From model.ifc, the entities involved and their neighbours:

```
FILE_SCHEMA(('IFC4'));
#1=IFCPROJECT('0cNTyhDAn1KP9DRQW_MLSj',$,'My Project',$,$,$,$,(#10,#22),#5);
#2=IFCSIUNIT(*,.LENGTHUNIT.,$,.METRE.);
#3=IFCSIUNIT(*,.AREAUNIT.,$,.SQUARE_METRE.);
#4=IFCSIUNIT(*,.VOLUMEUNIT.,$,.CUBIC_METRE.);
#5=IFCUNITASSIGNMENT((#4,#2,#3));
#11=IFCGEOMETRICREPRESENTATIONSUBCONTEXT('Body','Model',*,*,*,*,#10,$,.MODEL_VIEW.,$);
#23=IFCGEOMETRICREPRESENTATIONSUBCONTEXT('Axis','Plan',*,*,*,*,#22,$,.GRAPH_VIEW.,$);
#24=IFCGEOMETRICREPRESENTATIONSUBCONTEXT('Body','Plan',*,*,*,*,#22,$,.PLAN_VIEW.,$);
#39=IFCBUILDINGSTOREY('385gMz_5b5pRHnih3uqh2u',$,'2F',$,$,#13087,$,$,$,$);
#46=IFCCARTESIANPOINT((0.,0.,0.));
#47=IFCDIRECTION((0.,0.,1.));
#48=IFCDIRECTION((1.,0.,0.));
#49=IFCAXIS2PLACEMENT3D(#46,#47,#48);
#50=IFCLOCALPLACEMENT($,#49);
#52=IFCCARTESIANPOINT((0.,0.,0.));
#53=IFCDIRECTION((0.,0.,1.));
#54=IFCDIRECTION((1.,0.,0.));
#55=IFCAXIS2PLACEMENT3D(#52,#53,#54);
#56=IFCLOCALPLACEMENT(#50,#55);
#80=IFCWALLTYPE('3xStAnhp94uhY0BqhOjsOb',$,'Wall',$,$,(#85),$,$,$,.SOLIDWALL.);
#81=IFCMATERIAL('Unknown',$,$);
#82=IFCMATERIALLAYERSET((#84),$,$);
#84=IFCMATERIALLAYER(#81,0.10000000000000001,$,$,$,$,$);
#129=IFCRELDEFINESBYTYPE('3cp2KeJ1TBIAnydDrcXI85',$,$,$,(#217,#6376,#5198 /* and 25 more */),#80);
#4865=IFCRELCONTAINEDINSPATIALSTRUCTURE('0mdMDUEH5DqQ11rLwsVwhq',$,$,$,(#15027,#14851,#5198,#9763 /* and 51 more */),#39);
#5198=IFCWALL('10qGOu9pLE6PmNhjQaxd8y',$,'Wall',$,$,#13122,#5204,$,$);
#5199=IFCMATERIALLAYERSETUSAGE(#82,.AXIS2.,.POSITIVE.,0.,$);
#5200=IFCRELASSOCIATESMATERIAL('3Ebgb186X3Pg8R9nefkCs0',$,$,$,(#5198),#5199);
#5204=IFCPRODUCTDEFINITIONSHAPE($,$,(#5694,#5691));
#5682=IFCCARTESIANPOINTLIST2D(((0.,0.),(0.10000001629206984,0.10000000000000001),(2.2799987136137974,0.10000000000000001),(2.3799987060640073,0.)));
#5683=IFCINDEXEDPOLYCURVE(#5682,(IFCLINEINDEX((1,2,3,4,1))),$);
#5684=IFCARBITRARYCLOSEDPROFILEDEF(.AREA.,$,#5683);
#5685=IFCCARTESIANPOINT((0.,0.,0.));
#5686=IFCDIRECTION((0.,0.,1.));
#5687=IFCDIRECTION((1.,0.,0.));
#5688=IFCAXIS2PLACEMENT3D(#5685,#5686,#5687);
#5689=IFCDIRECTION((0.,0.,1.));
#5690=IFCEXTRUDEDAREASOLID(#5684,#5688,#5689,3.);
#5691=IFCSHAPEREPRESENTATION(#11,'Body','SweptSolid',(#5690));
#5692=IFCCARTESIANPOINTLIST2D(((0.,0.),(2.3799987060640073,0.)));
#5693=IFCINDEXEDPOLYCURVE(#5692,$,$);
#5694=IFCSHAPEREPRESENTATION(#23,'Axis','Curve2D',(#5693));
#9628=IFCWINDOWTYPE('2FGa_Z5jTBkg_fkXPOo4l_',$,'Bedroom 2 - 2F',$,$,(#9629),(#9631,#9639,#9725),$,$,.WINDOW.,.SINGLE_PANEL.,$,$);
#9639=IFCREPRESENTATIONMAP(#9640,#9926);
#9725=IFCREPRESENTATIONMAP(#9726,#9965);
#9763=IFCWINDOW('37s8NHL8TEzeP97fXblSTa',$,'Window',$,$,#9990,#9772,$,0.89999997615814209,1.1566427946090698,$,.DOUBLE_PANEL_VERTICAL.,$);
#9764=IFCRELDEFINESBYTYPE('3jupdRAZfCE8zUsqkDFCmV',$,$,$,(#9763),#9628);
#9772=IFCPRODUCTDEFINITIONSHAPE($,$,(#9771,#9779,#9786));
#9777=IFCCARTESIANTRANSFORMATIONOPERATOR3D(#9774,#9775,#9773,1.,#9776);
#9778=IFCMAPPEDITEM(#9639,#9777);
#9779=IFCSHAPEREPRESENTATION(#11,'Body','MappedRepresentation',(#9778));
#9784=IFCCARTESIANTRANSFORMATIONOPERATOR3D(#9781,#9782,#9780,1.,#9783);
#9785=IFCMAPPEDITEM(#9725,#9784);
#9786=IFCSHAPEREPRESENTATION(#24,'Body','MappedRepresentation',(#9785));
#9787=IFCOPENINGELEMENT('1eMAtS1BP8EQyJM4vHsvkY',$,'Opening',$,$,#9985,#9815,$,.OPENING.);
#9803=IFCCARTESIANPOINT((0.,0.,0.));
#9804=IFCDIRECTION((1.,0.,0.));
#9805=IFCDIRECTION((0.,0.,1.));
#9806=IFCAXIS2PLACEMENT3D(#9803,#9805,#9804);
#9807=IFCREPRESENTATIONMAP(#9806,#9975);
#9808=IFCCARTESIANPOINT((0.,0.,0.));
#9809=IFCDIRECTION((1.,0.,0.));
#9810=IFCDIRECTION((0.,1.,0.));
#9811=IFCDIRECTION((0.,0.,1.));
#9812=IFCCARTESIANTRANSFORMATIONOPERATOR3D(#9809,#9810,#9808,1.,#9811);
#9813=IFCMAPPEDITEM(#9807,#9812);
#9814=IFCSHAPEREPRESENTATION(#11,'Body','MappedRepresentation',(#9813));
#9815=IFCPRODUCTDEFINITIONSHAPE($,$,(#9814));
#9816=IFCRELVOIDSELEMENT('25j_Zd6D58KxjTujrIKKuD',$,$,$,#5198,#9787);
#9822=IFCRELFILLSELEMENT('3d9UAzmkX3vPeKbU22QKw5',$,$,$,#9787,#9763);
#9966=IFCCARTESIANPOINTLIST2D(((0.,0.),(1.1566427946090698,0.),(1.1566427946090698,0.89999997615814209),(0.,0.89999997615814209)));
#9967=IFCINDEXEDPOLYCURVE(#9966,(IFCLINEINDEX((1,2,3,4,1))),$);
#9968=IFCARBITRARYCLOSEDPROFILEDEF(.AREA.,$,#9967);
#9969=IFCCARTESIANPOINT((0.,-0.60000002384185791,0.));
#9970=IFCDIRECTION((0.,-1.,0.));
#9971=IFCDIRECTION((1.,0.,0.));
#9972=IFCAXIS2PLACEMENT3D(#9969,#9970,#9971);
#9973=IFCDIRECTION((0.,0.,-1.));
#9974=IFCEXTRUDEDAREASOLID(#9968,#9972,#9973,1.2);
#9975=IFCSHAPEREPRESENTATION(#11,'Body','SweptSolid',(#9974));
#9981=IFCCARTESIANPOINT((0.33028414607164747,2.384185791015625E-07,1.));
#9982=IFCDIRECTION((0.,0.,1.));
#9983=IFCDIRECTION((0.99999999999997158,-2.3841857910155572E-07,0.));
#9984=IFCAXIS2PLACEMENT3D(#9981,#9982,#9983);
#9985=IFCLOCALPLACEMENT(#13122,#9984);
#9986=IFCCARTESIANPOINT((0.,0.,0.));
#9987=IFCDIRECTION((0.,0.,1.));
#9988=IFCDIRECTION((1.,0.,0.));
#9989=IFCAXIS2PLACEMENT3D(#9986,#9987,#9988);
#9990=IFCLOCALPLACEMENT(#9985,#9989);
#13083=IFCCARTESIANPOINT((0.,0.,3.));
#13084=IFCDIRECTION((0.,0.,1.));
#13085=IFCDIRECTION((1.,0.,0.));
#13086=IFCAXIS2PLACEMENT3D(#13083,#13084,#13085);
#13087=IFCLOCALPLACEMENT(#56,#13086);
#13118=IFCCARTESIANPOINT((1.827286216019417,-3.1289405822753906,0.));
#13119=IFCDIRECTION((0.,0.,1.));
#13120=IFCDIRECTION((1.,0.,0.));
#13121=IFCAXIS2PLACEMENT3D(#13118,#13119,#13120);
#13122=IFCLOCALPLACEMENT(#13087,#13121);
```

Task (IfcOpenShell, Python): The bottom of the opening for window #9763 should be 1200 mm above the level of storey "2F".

```python
import numpy as np
import ifcopenshell
import ifcopenshell.api.geometry
import ifcopenshell.geom
import ifcopenshell.util.element
import ifcopenshell.util.placement
import ifcopenshell.util.shape
import ifcopenshell.util.unit

model = ifcopenshell.open("model.ifc")
unit_scale = ifcopenshell.util.unit.calculate_unit_scale(model)

window = model.by_guid("37s8NHL8TEzeP97fXblSTa")
opening = window.FillsVoids[0].RelatingOpeningElement
storey = ifcopenshell.util.element.get_container(window, ifc_class="IfcBuildingStorey")
level = ifcopenshell.util.placement.get_local_placement(storey.ObjectPlacement)[2, 3]

# The opening's origin need not be at the sill, so measure its lowest point.
shape = ifcopenshell.geom.create_shape(ifcopenshell.geom.settings(), opening)
bottom = ifcopenshell.util.shape.get_shape_bottom_elevation(shape, shape.geometry) / unit_scale
dz = level + 1.2 / unit_scale - bottom

shift = np.array([0.0, 0.0, dz])
# The window is placed relative to its opening, so it follows when the opening moves.
matrix = ifcopenshell.util.placement.get_local_placement(opening.ObjectPlacement)
matrix[:3, 3] += shift
ifcopenshell.api.geometry.edit_object_placement(
    model, product=opening, matrix=matrix, is_si=False, should_transform_children=True
)

print(f"moved by {dz * unit_scale:+.3f} m")

model.write("model_rev.ifc")
```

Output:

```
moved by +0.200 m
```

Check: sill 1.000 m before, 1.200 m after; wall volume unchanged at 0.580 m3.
